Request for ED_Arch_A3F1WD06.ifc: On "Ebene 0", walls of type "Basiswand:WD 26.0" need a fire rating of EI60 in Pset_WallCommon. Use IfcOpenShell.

First a look at what the model holds.

```python
import ifcopenshell
import ifcopenshell.util.element

model = ifcopenshell.open("ED_Arch_A3F1WD06.ifc")
print(model.schema)
storey = next(s for s in model.by_type("IfcBuildingStorey") if s.Name == "Ebene 0")
walls = [e for e in ifcopenshell.util.element.get_decomposition(storey) if e.is_a("IfcWall")]
seen = {}
for e in walls:
    element_type = ifcopenshell.util.element.get_type(e)
    key = (element_type.Name if element_type != e and element_type else None, ifcopenshell.util.element.get_pset(e, "Pset_WallCommon", "FireRating"))
    seen[key] = seen.get(key, 0) + 1
for (name, value), count in sorted(seen.items(), key=str):
    print(count, "x", name, "|", value)
```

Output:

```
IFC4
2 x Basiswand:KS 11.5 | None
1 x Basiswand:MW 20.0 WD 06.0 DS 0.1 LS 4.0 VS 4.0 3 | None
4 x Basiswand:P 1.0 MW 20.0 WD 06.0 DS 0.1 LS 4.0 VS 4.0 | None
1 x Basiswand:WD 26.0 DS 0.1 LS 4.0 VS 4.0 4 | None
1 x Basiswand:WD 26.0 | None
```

```python
import ifcopenshell
import ifcopenshell.api.pset
import ifcopenshell.util.element

model = ifcopenshell.open("ED_Arch_A3F1WD06.ifc")

storey = next(s for s in model.by_type("IfcBuildingStorey") if s.Name == "Ebene 0")
walls = [e for e in ifcopenshell.util.element.get_decomposition(storey) if e.is_a("IfcWall")]

count = 0
for e in walls:
    element_type = ifcopenshell.util.element.get_type(e)
    if element_type in (None, e) or element_type.Name != "Basiswand:WD 26.0":
        continue
    # add_pset returns the element's existing set when there is one.
    pset = ifcopenshell.api.pset.add_pset(model, product=e, name="Pset_WallCommon")
    ifcopenshell.api.pset.edit_pset(model, pset=pset, properties={"FireRating": "EI60"})
    count += 1

print(count, "walls updated")

model.write("ED_Arch_A3F1WD06_updated.ifc")
```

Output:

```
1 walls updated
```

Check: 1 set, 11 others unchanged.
